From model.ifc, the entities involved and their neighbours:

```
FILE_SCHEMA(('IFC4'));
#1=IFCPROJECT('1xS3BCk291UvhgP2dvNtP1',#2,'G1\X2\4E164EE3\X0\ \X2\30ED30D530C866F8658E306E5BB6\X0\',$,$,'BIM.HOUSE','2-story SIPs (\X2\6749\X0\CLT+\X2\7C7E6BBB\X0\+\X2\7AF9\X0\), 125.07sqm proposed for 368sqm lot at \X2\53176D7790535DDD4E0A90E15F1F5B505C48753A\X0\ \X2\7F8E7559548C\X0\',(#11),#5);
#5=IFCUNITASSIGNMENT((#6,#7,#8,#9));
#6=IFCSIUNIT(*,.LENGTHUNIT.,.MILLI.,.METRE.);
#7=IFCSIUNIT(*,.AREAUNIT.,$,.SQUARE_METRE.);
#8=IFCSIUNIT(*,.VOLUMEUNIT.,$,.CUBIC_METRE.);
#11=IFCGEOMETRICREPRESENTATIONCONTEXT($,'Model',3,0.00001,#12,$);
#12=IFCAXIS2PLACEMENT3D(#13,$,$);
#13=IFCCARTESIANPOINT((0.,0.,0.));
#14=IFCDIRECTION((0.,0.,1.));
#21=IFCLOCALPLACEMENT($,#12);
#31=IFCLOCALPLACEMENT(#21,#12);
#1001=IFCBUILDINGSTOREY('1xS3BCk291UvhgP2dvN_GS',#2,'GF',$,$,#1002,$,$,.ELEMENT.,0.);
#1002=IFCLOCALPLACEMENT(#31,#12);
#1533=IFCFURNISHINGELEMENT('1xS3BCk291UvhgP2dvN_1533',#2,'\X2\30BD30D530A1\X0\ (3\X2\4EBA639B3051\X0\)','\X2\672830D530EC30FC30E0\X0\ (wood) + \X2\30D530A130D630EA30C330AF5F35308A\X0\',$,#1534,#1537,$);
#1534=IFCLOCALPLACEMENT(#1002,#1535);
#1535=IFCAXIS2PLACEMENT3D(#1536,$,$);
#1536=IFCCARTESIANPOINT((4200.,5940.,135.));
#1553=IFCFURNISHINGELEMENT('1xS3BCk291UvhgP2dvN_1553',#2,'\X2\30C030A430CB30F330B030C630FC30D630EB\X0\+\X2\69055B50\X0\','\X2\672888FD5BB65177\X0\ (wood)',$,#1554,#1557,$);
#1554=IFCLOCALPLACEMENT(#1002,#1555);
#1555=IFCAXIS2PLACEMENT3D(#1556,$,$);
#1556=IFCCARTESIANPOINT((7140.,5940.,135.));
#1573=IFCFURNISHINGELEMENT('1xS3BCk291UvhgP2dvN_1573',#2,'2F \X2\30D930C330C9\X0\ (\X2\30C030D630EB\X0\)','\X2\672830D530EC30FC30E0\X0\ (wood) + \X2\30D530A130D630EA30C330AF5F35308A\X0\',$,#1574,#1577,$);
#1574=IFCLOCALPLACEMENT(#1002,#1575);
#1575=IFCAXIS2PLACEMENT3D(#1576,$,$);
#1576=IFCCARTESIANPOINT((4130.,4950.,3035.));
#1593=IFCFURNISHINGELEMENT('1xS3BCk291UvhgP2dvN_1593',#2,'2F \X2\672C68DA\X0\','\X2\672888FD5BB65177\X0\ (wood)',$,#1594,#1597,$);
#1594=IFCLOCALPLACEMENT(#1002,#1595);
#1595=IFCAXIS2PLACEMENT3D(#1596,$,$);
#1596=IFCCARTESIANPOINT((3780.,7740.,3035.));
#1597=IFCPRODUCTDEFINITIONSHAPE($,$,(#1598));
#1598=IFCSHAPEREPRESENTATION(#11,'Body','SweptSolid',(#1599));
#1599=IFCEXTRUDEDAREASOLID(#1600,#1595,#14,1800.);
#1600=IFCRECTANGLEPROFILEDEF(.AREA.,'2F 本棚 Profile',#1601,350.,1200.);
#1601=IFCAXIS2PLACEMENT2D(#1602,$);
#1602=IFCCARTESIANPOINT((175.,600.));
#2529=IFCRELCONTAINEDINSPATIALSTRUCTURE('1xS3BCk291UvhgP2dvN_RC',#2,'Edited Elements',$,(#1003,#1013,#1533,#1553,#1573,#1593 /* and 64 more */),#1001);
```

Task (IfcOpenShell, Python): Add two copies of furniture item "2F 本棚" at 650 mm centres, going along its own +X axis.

```python
import ifcopenshell
import ifcopenshell.api.geometry
import ifcopenshell.api.root
import ifcopenshell.util.element
import ifcopenshell.util.placement

model = ifcopenshell.open("model.ifc")


def reuse_history(source, copy):
    """copy_class also copies each property set's owner history, people and application; keep the originals."""
    for rel in copy.IsDefinedBy:
        if rel.is_a("IfcRelDefinesByProperties") and (history := rel.RelatingPropertyDefinition.OwnerHistory):
            rel.RelatingPropertyDefinition.OwnerHistory = source.OwnerHistory
            ifcopenshell.util.element.remove_deep2(model, history)


source = model.by_guid("1xS3BCk291UvhgP2dvN_1593")
base = ifcopenshell.util.placement.get_local_placement(source.ObjectPlacement)
step = base[:3, 0] * 650.0

for i in range(1, 3):
    copy = ifcopenshell.api.root.copy_class(model, product=source)
    copy.Representation = ifcopenshell.util.element.copy_deep(
        model, source.Representation, exclude=["IfcGeometricRepresentationContext", "IfcRepresentationMap"]
    )
    reuse_history(source, copy)
    matrix = base.copy()
    matrix[:3, 3] += i * step
    print("added at", matrix[:3, 3].round(3) + 0.0)
    ifcopenshell.api.geometry.edit_object_placement(model, product=copy, matrix=matrix, is_si=False)

model.write("model_v2.ifc")
```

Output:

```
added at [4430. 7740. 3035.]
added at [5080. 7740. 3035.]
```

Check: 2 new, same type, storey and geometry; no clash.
